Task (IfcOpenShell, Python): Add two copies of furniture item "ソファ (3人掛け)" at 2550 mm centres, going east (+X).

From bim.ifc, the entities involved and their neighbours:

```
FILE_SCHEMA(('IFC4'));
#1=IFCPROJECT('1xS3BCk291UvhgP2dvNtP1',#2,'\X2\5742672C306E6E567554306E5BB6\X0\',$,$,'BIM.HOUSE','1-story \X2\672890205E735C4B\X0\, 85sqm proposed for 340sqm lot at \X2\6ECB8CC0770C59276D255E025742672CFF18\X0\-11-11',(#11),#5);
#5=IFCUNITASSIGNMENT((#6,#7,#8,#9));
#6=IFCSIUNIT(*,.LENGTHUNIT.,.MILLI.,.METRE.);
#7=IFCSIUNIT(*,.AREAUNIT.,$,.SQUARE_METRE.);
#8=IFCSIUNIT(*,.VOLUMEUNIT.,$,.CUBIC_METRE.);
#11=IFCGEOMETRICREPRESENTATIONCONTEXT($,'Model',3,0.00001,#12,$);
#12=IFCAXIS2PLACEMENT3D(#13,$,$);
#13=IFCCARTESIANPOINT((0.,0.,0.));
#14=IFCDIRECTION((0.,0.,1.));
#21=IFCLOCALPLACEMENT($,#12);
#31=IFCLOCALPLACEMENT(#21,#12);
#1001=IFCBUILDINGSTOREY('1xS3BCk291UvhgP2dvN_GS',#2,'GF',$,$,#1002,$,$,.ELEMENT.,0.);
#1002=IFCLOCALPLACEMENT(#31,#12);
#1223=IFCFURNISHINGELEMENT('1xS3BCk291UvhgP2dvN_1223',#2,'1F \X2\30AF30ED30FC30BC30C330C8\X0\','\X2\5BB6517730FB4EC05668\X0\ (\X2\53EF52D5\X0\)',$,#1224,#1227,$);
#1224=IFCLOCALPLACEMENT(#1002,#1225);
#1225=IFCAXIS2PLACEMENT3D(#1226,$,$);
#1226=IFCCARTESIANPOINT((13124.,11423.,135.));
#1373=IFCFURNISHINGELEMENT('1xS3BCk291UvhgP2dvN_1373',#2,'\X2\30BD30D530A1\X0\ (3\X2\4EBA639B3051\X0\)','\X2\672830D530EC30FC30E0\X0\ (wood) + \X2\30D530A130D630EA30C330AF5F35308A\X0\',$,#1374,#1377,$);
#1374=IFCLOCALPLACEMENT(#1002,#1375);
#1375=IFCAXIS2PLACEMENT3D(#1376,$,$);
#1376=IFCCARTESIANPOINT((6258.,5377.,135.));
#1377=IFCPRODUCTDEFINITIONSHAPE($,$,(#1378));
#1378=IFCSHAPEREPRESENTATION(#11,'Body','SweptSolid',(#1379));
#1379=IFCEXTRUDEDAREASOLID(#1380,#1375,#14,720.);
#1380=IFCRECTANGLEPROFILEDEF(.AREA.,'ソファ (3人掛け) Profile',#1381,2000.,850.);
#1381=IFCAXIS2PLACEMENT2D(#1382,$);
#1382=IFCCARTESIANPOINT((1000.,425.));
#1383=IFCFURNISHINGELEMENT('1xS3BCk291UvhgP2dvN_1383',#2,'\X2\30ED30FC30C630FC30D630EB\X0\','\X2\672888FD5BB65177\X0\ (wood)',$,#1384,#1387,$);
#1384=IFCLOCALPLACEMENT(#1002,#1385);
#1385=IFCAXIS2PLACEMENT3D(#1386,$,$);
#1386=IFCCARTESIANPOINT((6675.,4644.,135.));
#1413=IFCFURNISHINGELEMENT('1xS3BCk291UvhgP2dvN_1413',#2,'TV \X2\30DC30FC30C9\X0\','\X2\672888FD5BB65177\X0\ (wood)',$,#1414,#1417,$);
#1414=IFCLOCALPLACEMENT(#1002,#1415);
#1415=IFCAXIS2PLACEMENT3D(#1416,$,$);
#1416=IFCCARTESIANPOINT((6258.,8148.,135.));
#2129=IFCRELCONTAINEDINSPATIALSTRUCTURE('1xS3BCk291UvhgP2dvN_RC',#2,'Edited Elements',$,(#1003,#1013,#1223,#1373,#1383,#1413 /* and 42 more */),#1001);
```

```python
import numpy as np
import ifcopenshell
import ifcopenshell.api.geometry
import ifcopenshell.api.root
import ifcopenshell.util.element
import ifcopenshell.util.placement
import ifcopenshell.util.unit

model = ifcopenshell.open("bim.ifc")
unit_scale = ifcopenshell.util.unit.calculate_unit_scale(model)


def reuse_history(source, copy):
    """copy_class also copies each property set's owner history, people and application; keep the originals."""
    for rel in copy.IsDefinedBy:
        if rel.is_a("IfcRelDefinesByProperties") and (history := rel.RelatingPropertyDefinition.OwnerHistory):
            rel.RelatingPropertyDefinition.OwnerHistory = source.OwnerHistory
            ifcopenshell.util.element.remove_deep2(model, history)


source = model.by_guid("1xS3BCk291UvhgP2dvN_1373")
base = ifcopenshell.util.placement.get_local_placement(source.ObjectPlacement)
step = np.array([1.0, 0.0, 0.0]) * 2.55 / unit_scale

for i in range(1, 3):
    copy = ifcopenshell.api.root.copy_class(model, product=source)
    copy.Representation = ifcopenshell.util.element.copy_deep(
        model, source.Representation, exclude=["IfcGeometricRepresentationContext", "IfcRepresentationMap"]
    )
    reuse_history(source, copy)
    matrix = base.copy()
    matrix[:3, 3] += i * step
    print("added at", matrix[:3, 3].round(3) + 0.0)
    ifcopenshell.api.geometry.edit_object_placement(model, product=copy, matrix=matrix, is_si=False)

model.write("bim_v2.ifc")
```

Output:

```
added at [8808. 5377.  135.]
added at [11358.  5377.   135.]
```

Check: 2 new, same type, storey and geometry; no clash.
